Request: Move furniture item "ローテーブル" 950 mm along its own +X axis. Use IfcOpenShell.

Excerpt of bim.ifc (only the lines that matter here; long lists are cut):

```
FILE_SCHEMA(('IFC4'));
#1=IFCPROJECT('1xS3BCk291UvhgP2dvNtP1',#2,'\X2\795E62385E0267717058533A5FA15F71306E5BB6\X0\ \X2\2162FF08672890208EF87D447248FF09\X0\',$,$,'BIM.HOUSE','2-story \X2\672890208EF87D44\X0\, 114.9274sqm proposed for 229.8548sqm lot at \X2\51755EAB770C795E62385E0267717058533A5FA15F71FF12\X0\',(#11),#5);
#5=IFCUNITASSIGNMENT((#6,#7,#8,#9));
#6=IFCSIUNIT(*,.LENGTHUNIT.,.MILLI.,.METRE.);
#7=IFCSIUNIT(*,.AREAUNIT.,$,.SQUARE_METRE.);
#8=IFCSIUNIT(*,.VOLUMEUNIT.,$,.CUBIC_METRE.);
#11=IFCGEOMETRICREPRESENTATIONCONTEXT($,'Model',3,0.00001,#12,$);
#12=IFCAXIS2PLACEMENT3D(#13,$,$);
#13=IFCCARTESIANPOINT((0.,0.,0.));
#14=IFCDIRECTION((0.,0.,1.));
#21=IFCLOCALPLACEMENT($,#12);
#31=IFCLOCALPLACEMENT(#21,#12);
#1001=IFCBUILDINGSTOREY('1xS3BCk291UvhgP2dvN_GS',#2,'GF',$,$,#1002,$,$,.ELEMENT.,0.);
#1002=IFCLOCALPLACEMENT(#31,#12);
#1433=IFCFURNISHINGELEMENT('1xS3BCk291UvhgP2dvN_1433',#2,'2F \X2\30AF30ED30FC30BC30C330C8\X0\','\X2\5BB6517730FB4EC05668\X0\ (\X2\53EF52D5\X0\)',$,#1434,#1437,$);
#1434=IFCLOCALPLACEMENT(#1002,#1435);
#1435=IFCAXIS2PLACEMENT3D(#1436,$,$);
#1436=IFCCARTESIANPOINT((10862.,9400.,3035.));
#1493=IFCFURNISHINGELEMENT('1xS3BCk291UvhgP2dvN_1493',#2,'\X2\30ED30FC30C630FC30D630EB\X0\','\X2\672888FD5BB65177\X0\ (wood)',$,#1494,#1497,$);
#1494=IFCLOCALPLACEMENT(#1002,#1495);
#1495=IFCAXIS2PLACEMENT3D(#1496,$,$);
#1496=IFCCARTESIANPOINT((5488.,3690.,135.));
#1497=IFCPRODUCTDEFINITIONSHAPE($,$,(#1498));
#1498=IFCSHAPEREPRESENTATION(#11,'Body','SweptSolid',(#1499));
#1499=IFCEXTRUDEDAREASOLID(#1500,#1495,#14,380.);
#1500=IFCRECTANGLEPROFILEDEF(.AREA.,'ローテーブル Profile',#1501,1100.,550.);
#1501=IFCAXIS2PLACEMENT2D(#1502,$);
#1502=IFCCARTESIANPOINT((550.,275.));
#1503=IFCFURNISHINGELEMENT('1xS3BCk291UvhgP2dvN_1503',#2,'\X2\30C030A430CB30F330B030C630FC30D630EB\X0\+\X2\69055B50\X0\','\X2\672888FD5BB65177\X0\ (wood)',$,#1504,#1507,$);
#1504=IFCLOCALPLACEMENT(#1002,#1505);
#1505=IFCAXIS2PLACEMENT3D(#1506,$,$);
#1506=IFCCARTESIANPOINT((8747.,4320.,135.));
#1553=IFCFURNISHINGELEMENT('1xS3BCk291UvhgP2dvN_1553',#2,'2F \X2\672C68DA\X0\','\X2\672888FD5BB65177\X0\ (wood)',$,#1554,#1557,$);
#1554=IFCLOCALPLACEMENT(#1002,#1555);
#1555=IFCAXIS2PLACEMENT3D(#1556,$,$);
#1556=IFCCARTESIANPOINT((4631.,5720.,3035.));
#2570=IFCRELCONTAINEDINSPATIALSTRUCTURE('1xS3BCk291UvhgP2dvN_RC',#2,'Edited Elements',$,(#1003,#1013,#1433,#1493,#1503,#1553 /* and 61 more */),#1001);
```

```python
import ifcopenshell
import ifcopenshell.api.geometry
import ifcopenshell.util.placement

model = ifcopenshell.open("bim.ifc")

item = model.by_guid("1xS3BCk291UvhgP2dvN_1493")
matrix = ifcopenshell.util.placement.get_local_placement(item.ObjectPlacement)
matrix[:3, 3] += matrix[:3, 0] * 950.0
ifcopenshell.api.geometry.edit_object_placement(model, product=item, matrix=matrix, is_si=False)

print(ifcopenshell.util.placement.get_local_placement(item.ObjectPlacement).round(3) + 0.0)

model.write("bim_v2.ifc")
```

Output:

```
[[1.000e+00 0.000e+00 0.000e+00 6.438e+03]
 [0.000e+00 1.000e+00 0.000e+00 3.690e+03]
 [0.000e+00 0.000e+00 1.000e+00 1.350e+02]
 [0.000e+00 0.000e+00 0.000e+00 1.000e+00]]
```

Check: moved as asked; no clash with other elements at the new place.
